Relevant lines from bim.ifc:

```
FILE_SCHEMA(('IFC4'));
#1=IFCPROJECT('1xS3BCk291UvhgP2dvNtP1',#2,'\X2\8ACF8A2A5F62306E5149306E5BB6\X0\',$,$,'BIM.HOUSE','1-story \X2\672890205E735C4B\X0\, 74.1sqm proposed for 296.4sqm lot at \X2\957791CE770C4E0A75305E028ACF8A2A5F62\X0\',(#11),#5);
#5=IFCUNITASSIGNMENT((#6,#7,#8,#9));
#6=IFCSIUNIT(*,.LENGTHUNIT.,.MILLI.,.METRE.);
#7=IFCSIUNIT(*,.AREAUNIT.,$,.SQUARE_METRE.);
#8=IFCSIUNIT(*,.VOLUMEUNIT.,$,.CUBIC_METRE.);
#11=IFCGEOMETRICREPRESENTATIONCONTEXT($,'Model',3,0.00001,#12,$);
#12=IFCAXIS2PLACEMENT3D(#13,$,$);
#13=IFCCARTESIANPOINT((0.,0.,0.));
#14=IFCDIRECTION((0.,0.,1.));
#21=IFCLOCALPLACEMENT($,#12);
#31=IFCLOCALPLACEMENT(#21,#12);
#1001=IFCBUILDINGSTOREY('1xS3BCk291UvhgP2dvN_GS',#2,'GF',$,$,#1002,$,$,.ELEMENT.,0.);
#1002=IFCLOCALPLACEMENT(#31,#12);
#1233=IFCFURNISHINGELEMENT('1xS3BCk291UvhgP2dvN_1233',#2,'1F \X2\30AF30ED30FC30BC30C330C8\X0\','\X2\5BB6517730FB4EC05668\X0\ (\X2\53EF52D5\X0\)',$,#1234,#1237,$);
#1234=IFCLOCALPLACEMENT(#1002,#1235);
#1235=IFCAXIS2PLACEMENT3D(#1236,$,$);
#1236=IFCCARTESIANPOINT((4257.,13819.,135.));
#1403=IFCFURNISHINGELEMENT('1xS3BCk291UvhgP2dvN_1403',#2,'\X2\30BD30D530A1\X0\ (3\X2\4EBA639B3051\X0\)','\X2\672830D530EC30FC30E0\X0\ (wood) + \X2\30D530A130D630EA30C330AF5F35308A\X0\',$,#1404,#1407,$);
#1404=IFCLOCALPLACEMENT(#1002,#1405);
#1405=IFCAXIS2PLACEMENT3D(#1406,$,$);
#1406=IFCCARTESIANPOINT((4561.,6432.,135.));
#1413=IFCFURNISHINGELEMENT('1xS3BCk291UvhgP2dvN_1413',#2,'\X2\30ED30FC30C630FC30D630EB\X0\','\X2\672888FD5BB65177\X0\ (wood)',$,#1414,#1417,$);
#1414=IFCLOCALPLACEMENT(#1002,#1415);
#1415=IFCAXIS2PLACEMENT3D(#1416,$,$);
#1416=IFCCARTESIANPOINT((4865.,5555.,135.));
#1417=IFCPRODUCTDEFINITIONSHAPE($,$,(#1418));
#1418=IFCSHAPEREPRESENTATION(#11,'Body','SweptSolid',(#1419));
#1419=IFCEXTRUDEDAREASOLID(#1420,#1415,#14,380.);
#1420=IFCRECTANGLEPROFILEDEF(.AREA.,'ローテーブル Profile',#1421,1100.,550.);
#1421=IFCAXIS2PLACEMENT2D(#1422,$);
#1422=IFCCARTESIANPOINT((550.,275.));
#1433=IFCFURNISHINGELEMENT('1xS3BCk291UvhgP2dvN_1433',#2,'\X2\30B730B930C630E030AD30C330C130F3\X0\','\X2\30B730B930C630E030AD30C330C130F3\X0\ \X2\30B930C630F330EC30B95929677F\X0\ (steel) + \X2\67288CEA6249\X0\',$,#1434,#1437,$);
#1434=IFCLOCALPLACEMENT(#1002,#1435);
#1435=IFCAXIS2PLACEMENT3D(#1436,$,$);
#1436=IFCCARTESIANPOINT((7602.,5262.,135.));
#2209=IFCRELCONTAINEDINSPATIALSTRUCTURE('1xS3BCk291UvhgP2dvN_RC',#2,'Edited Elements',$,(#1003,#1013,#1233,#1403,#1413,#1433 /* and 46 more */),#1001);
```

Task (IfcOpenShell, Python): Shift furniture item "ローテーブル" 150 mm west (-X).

```python
import ifcopenshell
import ifcopenshell.api.geometry
import ifcopenshell.util.placement

model = ifcopenshell.open("bim.ifc")

item = model.by_guid("1xS3BCk291UvhgP2dvN_1413")
matrix = ifcopenshell.util.placement.get_local_placement(item.ObjectPlacement)
matrix[0, 3] -= 150.0
ifcopenshell.api.geometry.edit_object_placement(model, product=item, matrix=matrix, is_si=False)

print(ifcopenshell.util.placement.get_local_placement(item.ObjectPlacement).round(3) + 0.0)

model.write("bim_edited.ifc")
```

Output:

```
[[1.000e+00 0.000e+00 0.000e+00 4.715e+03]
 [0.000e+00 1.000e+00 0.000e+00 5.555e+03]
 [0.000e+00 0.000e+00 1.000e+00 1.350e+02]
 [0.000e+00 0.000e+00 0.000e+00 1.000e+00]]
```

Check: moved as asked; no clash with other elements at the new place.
